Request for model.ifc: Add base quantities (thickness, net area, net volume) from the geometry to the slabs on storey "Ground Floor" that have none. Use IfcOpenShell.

First a look at what the model holds.

```python
import ifcopenshell
import ifcopenshell.util.element
import ifcopenshell.util.unit

model = ifcopenshell.open("model.ifc")
print(model.schema)
for unit_type in ("LENGTHUNIT", "AREAUNIT", "VOLUMEUNIT"):
    print(unit_type, ifcopenshell.util.unit.calculate_unit_scale(model, unit_type))
storey = next(s for s in model.by_type("IfcBuildingStorey") if s.Name == "Ground Floor")
slabs = [e for e in ifcopenshell.util.element.get_decomposition(storey) if e.is_a("IfcSlab")]
for e in sorted(slabs, key=lambda e: e.id()):
    print(e.id(), e.is_a(), e.Name, list(ifcopenshell.util.element.get_psets(e, qtos_only=True)), sep=" | ")
```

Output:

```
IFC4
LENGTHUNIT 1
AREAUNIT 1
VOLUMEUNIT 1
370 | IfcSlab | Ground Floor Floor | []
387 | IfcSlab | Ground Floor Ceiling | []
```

```python
import ifcopenshell
import ifcopenshell.api.pset
import ifcopenshell.geom
import ifcopenshell.util.element
import ifcopenshell.util.shape
import ifcopenshell.util.unit

model = ifcopenshell.open("model.ifc")
unit_scale = ifcopenshell.util.unit.calculate_unit_scale(model)
area_scale = ifcopenshell.util.unit.calculate_unit_scale(model, "AREAUNIT")
volume_scale = ifcopenshell.util.unit.calculate_unit_scale(model, "VOLUMEUNIT")
settings = ifcopenshell.geom.settings()

storey = next(s for s in model.by_type("IfcBuildingStorey") if s.Name == "Ground Floor")
slabs = [e for e in ifcopenshell.util.element.get_decomposition(storey) if e.is_a("IfcSlab")]

for e in sorted(slabs, key=lambda e: e.id()):
    if ifcopenshell.util.element.get_psets(e, qtos_only=True, should_inherit=False):
        continue
    # Geometry comes back in metres, in the element's own axes.
    shape = ifcopenshell.geom.create_shape(settings, e)
    values = {
        "Width": ifcopenshell.util.shape.get_z(shape.geometry) / unit_scale,
        "NetArea": ifcopenshell.util.shape.get_footprint_area(shape.geometry) / area_scale,
        "NetVolume": ifcopenshell.util.shape.get_volume(shape.geometry) / volume_scale,
    }
    qto = ifcopenshell.api.pset.add_qto(model, product=e, name="Qto_SlabBaseQuantities")
    ifcopenshell.api.pset.edit_qto(model, qto=qto, properties=values)
    print(e.id(), {k: round(v, 3) for k, v in values.items()})

model.write("model_v2.ifc")
```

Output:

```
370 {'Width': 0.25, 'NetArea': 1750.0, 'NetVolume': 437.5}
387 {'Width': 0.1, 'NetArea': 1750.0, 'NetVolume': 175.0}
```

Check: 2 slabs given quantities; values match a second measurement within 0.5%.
